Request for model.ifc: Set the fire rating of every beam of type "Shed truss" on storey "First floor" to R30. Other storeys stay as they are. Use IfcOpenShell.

First a look at what the model holds.

```python
import ifcopenshell
import ifcopenshell.util.element

model = ifcopenshell.open("model.ifc")
print(model.schema)
storey = next(s for s in model.by_type("IfcBuildingStorey") if s.Name == "First floor")
beams = [e for e in ifcopenshell.util.element.get_decomposition(storey) if e.is_a("IfcBeam")]
seen = {}
for e in beams:
    element_type = ifcopenshell.util.element.get_type(e)
    key = (element_type.Name if element_type != e and element_type else None, ifcopenshell.util.element.get_pset(e, "Pset_BeamCommon", "FireRating"))
    seen[key] = seen.get(key, 0) + 1
for (name, value), count in sorted(seen.items(), key=str):
    print(count, "x", name, "|", value)
```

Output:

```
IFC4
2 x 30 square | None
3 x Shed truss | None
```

```python
import ifcopenshell
import ifcopenshell.api.pset
import ifcopenshell.util.element

model = ifcopenshell.open("model.ifc")

storey = next(s for s in model.by_type("IfcBuildingStorey") if s.Name == "First floor")
beams = [e for e in ifcopenshell.util.element.get_decomposition(storey) if e.is_a("IfcBeam")]

count = 0
for e in beams:
    element_type = ifcopenshell.util.element.get_type(e)
    if element_type in (None, e) or element_type.Name != "Shed truss":
        continue
    # add_pset returns the element's existing set when there is one.
    pset = ifcopenshell.api.pset.add_pset(model, product=e, name="Pset_BeamCommon")
    ifcopenshell.api.pset.edit_pset(model, pset=pset, properties={"FireRating": "R30"})
    count += 1

print(count, "beams updated")

model.write("model_updated.ifc")
```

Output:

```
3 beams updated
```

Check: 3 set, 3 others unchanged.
